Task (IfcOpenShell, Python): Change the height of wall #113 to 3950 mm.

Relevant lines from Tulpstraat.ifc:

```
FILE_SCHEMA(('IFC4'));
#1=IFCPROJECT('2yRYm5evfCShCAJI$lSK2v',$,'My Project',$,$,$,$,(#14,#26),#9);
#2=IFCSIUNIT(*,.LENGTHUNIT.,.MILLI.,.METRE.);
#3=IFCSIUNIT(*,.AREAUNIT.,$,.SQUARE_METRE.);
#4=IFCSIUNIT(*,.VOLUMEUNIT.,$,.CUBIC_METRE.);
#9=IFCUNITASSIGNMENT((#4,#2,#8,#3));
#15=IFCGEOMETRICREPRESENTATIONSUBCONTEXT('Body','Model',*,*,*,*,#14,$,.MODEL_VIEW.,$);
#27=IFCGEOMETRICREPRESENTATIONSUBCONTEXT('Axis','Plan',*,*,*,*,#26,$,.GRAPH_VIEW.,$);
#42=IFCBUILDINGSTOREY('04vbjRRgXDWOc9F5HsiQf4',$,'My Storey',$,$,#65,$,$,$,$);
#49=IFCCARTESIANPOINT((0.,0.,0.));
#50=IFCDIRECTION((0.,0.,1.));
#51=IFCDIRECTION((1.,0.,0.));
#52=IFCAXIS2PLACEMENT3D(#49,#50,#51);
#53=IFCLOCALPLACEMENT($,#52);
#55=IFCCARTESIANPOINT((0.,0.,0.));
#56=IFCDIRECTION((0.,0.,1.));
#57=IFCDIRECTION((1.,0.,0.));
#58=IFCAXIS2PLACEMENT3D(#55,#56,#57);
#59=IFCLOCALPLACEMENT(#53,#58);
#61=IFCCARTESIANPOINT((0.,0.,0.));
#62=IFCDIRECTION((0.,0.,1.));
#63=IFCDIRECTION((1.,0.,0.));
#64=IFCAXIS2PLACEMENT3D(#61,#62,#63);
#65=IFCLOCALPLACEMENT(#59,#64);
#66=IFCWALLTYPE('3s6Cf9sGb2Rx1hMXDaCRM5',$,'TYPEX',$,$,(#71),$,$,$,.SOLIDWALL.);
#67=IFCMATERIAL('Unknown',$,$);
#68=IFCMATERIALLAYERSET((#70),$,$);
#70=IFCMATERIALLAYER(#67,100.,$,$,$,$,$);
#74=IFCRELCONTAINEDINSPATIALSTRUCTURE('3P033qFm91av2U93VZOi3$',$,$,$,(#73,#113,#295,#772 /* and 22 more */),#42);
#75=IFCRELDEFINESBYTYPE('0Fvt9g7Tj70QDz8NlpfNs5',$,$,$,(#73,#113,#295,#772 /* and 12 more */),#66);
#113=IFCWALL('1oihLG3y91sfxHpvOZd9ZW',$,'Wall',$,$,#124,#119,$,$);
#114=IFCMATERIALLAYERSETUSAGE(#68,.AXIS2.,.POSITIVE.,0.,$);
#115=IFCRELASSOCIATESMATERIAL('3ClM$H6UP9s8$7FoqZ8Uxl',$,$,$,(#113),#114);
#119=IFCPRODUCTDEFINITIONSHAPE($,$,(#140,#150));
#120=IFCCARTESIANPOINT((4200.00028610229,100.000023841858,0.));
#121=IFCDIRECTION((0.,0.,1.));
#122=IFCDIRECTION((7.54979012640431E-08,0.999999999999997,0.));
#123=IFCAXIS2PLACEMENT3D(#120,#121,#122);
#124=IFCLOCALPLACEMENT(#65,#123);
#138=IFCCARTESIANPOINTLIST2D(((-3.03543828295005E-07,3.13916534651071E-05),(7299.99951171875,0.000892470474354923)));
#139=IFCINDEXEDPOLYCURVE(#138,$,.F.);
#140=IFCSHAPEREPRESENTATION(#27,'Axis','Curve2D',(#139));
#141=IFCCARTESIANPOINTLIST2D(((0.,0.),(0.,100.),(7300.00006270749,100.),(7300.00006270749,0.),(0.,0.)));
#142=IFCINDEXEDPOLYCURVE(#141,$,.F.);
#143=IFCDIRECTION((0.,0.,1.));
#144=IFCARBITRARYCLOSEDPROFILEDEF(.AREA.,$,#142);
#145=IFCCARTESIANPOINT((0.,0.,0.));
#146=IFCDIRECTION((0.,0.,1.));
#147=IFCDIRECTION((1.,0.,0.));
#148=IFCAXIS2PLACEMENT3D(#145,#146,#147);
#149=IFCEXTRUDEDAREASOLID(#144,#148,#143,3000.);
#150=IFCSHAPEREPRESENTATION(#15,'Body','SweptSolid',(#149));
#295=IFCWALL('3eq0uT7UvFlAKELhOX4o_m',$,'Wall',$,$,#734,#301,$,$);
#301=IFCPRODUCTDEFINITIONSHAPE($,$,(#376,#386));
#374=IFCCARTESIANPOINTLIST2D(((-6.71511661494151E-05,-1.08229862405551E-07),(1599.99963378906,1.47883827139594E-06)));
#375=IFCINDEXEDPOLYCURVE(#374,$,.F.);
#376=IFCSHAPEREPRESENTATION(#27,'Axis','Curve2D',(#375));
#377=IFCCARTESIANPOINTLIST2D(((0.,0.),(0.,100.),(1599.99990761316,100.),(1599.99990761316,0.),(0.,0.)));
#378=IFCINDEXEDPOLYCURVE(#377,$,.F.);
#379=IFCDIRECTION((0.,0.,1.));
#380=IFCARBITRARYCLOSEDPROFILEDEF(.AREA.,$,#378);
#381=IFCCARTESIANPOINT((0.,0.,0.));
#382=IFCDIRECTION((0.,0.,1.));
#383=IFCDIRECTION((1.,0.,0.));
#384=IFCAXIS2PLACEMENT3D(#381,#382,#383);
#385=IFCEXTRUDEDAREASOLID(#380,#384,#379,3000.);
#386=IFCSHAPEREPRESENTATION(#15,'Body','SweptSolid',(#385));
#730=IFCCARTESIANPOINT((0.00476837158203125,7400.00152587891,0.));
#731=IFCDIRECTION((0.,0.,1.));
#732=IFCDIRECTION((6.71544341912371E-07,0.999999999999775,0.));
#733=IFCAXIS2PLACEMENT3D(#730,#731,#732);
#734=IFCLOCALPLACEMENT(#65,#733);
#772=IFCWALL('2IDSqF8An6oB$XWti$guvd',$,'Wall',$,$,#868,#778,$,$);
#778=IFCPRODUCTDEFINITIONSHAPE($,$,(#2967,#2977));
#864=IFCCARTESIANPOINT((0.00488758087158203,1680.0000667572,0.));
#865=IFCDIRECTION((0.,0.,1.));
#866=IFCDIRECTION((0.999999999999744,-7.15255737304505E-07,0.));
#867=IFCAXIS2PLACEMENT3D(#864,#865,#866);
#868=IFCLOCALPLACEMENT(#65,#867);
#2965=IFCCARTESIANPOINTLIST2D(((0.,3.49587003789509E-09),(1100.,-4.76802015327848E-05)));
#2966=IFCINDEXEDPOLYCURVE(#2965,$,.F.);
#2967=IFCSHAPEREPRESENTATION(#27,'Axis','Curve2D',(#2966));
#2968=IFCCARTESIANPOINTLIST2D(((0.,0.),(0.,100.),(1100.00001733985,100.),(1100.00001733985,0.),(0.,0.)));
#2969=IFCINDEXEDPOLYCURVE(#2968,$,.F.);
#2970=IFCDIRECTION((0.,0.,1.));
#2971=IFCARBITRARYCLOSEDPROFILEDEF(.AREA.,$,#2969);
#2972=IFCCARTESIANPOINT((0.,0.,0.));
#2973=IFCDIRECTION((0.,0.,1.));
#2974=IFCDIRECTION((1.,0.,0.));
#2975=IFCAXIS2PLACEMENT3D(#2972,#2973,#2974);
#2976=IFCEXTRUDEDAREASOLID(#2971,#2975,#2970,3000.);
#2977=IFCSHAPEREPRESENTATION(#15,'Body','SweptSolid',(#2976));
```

```python
import ifcopenshell
import ifcopenshell.geom
import ifcopenshell.util.representation
import ifcopenshell.util.shape
import ifcopenshell.util.unit

model = ifcopenshell.open("Tulpstraat.ifc")
unit_scale = ifcopenshell.util.unit.calculate_unit_scale(model)
settings = ifcopenshell.geom.settings()


def volume(element):
    """Net volume in cubic metres, openings subtracted."""
    shape = ifcopenshell.geom.create_shape(settings, element)
    return ifcopenshell.util.shape.get_volume(shape.geometry)


wall = model.by_guid("1oihLG3y91sfxHpvOZd9ZW")
before = volume(wall)

body = ifcopenshell.util.representation.get_representation(wall, "Model", "Body")
solid = body.Items[0]
old_height = solid.Depth
solid.Depth = 3.95 / unit_scale
after = volume(wall)

print(f"height {old_height:g} -> {solid.Depth:g}, volume {before:.3f} -> {after:.3f} m3")

model.write("Tulpstraat_updated.ifc")
```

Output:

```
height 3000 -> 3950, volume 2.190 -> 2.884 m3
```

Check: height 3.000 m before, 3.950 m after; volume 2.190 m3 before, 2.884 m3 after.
